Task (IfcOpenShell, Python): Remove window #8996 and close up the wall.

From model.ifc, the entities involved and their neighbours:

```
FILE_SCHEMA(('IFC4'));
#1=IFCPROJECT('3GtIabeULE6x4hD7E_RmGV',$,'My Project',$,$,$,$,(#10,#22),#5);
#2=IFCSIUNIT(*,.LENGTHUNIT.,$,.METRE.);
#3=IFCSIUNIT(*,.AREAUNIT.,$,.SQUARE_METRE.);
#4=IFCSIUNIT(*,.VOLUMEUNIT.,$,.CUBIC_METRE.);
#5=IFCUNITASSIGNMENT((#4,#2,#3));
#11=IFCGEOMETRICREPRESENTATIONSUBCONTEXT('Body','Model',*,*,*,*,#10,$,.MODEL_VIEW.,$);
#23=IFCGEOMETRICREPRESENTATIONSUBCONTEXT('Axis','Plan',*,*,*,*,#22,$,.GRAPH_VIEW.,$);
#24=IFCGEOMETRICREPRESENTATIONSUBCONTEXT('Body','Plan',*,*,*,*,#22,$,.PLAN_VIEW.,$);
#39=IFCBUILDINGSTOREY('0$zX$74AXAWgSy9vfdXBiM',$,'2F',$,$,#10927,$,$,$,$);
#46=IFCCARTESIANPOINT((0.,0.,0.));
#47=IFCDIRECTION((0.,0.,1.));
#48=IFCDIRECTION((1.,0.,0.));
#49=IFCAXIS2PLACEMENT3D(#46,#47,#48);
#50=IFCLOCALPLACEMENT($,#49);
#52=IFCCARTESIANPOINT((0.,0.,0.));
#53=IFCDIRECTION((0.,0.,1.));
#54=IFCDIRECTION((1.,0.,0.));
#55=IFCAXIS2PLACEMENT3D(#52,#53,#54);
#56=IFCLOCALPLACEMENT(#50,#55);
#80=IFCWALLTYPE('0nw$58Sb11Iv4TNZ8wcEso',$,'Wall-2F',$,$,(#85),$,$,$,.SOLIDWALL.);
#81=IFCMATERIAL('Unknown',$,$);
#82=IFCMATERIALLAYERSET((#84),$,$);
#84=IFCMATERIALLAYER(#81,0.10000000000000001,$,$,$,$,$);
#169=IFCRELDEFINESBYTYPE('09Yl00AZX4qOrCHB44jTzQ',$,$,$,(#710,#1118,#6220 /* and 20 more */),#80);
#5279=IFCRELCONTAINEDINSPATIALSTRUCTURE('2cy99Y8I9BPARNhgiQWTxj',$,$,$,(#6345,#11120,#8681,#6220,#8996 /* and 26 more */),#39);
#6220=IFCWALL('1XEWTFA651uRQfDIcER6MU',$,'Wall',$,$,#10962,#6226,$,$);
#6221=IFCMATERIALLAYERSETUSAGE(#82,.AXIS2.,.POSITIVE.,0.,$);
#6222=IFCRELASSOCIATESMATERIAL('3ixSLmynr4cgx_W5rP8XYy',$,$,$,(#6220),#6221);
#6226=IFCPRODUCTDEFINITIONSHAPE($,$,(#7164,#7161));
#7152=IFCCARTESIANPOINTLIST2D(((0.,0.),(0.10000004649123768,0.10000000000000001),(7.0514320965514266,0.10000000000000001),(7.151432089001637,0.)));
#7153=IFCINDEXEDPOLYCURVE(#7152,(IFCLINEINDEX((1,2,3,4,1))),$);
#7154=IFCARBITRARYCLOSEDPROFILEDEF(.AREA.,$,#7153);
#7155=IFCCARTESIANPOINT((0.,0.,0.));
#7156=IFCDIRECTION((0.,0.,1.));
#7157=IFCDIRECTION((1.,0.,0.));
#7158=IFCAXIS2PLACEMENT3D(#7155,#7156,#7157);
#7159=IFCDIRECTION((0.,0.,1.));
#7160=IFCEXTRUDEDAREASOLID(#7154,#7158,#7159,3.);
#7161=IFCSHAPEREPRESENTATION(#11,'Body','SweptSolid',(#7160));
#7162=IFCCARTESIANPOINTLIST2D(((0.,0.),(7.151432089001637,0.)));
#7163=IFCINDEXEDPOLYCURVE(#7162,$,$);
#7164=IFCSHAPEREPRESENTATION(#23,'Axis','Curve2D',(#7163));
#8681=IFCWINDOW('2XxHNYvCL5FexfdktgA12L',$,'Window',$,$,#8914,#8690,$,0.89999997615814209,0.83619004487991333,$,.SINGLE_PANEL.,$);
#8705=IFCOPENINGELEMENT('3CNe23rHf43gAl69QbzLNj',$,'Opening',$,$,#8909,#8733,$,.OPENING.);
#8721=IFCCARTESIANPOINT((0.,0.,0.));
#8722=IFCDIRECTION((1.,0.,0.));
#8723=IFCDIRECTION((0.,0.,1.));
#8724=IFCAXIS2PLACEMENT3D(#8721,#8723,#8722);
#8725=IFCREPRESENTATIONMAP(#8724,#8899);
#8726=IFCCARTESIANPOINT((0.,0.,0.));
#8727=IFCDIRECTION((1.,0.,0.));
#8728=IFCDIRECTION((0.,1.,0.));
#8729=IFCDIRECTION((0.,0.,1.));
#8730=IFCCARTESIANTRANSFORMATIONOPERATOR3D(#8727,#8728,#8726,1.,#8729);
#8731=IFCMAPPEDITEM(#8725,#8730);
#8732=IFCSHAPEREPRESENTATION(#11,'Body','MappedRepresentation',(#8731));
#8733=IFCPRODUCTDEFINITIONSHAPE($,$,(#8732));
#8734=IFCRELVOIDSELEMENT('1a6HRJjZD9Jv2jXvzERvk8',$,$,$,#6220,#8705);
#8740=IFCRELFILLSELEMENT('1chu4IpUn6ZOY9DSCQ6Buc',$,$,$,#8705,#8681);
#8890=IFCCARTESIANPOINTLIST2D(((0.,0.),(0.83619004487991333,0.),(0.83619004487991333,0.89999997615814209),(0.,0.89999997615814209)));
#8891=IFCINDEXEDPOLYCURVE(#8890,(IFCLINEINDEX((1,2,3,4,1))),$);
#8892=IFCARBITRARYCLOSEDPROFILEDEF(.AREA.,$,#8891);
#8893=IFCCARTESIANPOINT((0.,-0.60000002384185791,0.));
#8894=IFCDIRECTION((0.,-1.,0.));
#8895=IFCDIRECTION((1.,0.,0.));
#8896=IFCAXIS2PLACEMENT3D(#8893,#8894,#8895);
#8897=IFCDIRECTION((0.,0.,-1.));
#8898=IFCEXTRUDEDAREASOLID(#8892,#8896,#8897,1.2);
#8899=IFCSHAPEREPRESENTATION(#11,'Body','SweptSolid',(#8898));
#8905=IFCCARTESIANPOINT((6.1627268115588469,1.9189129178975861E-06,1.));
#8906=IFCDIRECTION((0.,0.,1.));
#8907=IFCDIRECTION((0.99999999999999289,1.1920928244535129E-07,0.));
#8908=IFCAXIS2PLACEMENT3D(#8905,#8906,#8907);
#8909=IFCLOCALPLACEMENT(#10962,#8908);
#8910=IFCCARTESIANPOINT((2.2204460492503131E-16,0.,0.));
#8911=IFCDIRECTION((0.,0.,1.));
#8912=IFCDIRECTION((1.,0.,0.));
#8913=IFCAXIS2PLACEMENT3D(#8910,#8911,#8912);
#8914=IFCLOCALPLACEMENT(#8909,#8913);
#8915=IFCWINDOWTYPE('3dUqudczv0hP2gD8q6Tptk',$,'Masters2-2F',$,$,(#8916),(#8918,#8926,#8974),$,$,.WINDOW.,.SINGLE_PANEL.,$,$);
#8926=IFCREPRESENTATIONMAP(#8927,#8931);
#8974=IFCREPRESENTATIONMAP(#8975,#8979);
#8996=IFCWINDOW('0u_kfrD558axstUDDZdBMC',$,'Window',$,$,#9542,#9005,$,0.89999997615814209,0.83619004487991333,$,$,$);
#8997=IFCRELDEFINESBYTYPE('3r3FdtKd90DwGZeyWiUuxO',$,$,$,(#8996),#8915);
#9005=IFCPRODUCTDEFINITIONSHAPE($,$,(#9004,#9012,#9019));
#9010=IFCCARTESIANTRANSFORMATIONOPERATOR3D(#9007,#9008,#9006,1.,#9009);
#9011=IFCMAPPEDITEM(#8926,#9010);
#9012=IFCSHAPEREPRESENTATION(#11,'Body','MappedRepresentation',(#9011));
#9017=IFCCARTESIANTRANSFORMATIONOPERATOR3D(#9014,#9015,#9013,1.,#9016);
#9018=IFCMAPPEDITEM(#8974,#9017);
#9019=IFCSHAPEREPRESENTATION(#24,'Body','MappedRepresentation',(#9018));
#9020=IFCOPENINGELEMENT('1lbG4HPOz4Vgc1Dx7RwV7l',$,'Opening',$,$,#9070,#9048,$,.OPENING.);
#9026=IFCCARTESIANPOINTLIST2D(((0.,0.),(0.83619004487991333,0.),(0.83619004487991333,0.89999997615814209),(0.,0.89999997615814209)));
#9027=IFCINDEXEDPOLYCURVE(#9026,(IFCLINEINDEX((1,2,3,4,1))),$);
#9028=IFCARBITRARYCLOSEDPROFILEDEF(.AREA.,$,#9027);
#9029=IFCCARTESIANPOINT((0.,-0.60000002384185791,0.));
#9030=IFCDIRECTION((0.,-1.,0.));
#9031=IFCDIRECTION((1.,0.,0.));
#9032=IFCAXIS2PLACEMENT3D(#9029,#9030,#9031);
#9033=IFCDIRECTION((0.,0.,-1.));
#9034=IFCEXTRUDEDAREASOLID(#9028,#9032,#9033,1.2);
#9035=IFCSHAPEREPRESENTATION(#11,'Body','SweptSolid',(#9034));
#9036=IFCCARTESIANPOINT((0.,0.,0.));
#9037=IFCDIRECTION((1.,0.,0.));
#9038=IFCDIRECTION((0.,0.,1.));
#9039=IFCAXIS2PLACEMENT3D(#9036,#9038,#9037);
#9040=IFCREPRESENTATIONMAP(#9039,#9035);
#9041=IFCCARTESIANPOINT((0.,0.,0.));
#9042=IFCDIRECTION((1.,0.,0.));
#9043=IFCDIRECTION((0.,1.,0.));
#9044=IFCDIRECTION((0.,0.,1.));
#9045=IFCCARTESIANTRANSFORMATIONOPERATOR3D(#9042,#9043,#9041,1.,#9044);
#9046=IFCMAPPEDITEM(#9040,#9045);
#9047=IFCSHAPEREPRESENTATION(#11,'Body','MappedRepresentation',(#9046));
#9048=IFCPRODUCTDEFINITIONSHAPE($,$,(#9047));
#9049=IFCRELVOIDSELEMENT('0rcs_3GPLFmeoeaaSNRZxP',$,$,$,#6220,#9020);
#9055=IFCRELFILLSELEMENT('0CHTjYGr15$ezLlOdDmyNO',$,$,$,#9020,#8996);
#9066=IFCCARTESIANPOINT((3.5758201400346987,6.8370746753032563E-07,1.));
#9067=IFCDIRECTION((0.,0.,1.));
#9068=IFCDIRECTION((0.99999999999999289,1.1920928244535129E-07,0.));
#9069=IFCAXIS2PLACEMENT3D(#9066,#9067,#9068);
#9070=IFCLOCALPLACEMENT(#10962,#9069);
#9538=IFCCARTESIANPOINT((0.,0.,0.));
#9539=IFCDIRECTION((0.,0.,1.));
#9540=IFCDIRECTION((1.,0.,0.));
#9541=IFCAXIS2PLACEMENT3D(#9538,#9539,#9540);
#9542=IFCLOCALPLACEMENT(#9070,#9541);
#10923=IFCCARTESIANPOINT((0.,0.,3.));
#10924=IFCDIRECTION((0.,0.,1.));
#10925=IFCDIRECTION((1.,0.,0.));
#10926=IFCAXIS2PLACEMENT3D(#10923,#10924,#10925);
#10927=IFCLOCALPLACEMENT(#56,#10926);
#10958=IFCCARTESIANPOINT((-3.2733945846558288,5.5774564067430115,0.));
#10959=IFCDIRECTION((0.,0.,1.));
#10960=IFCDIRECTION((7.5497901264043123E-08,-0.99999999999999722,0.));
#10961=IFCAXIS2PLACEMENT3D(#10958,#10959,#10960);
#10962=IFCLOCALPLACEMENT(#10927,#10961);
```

```python
import ifcopenshell
import ifcopenshell.api.feature
import ifcopenshell.api.root
import ifcopenshell.geom
import ifcopenshell.util.shape

model = ifcopenshell.open("model.ifc")
settings = ifcopenshell.geom.settings()


def volume(element):
    """Net volume in cubic metres, openings subtracted."""
    shape = ifcopenshell.geom.create_shape(settings, element)
    return ifcopenshell.util.shape.get_volume(shape.geometry)


window = model.by_id(8996)
opening = window.FillsVoids[0].RelatingOpeningElement
wall = opening.VoidsElements[0].RelatingBuildingElement
before = volume(wall)

ifcopenshell.api.root.remove_product(model, product=window)
ifcopenshell.api.feature.remove_feature(model, feature=opening)

after = volume(wall)

print(f"wall volume {before:.3f} -> {after:.3f} m3")

model.write("model-out.ifc")
```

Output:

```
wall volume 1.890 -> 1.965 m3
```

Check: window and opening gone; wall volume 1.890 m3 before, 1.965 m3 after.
